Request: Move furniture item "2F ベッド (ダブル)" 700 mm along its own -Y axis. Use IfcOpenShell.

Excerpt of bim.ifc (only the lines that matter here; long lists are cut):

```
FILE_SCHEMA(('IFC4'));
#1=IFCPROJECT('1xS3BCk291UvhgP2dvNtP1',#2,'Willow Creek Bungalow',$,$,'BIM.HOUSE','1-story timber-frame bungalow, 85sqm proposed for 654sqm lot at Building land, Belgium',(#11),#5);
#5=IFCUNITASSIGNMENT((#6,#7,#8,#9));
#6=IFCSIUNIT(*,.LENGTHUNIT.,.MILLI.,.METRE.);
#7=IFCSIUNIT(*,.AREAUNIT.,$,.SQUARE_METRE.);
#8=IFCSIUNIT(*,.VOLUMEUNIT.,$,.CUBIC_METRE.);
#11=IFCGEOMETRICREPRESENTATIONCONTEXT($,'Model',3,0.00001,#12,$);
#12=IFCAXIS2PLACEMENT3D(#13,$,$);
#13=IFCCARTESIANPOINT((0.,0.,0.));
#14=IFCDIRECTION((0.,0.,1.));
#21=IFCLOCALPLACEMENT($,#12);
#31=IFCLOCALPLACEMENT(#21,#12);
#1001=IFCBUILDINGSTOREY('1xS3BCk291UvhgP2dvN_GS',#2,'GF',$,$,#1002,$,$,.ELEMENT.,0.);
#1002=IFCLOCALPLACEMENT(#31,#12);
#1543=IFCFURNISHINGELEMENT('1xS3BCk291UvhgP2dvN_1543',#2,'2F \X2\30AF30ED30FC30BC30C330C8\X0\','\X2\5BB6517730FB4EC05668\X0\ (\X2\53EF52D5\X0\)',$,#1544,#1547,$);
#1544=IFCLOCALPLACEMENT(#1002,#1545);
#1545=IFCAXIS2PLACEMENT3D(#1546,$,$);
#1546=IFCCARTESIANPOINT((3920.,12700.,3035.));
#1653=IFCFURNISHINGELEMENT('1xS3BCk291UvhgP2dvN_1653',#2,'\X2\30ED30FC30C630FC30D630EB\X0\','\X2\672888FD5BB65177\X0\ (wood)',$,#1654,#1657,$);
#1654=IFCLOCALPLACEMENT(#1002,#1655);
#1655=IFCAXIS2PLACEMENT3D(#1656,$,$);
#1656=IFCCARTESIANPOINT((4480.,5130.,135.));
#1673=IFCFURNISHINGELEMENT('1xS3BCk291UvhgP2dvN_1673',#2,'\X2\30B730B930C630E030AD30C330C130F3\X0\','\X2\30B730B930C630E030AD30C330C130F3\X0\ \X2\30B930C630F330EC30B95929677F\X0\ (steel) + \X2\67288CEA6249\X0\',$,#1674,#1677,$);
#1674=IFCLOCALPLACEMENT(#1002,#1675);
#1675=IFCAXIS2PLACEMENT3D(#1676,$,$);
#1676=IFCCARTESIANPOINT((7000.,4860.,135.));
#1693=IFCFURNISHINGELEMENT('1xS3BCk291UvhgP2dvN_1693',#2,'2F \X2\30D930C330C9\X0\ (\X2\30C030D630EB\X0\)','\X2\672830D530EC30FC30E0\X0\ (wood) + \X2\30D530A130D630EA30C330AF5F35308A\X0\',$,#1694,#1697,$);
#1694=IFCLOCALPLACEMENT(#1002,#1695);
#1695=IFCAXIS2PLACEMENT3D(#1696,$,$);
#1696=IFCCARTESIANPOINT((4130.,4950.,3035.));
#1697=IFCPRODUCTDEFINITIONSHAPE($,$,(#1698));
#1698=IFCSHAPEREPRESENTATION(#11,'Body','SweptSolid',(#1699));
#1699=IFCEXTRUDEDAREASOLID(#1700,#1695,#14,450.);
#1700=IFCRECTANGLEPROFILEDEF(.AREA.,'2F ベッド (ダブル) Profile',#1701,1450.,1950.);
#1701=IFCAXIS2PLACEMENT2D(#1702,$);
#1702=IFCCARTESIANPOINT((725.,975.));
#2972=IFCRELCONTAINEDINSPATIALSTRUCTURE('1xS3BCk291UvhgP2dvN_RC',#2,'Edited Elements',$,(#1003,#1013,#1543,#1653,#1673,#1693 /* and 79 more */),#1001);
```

```python
import ifcopenshell
import ifcopenshell.api.geometry
import ifcopenshell.util.placement
import ifcopenshell.util.unit

model = ifcopenshell.open("bim.ifc")
unit_scale = ifcopenshell.util.unit.calculate_unit_scale(model)

item = model.by_guid("1xS3BCk291UvhgP2dvN_1693")
matrix = ifcopenshell.util.placement.get_local_placement(item.ObjectPlacement)
matrix[:3, 3] -= matrix[:3, 1] * 0.7 / unit_scale
ifcopenshell.api.geometry.edit_object_placement(model, product=item, matrix=matrix, is_si=False)

print(ifcopenshell.util.placement.get_local_placement(item.ObjectPlacement).round(3) + 0.0)

model.write("bim_rev.ifc")
```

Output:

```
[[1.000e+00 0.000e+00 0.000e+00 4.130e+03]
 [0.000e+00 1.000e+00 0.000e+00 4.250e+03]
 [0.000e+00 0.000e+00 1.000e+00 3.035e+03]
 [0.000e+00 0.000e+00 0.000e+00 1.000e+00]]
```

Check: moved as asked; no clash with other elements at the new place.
